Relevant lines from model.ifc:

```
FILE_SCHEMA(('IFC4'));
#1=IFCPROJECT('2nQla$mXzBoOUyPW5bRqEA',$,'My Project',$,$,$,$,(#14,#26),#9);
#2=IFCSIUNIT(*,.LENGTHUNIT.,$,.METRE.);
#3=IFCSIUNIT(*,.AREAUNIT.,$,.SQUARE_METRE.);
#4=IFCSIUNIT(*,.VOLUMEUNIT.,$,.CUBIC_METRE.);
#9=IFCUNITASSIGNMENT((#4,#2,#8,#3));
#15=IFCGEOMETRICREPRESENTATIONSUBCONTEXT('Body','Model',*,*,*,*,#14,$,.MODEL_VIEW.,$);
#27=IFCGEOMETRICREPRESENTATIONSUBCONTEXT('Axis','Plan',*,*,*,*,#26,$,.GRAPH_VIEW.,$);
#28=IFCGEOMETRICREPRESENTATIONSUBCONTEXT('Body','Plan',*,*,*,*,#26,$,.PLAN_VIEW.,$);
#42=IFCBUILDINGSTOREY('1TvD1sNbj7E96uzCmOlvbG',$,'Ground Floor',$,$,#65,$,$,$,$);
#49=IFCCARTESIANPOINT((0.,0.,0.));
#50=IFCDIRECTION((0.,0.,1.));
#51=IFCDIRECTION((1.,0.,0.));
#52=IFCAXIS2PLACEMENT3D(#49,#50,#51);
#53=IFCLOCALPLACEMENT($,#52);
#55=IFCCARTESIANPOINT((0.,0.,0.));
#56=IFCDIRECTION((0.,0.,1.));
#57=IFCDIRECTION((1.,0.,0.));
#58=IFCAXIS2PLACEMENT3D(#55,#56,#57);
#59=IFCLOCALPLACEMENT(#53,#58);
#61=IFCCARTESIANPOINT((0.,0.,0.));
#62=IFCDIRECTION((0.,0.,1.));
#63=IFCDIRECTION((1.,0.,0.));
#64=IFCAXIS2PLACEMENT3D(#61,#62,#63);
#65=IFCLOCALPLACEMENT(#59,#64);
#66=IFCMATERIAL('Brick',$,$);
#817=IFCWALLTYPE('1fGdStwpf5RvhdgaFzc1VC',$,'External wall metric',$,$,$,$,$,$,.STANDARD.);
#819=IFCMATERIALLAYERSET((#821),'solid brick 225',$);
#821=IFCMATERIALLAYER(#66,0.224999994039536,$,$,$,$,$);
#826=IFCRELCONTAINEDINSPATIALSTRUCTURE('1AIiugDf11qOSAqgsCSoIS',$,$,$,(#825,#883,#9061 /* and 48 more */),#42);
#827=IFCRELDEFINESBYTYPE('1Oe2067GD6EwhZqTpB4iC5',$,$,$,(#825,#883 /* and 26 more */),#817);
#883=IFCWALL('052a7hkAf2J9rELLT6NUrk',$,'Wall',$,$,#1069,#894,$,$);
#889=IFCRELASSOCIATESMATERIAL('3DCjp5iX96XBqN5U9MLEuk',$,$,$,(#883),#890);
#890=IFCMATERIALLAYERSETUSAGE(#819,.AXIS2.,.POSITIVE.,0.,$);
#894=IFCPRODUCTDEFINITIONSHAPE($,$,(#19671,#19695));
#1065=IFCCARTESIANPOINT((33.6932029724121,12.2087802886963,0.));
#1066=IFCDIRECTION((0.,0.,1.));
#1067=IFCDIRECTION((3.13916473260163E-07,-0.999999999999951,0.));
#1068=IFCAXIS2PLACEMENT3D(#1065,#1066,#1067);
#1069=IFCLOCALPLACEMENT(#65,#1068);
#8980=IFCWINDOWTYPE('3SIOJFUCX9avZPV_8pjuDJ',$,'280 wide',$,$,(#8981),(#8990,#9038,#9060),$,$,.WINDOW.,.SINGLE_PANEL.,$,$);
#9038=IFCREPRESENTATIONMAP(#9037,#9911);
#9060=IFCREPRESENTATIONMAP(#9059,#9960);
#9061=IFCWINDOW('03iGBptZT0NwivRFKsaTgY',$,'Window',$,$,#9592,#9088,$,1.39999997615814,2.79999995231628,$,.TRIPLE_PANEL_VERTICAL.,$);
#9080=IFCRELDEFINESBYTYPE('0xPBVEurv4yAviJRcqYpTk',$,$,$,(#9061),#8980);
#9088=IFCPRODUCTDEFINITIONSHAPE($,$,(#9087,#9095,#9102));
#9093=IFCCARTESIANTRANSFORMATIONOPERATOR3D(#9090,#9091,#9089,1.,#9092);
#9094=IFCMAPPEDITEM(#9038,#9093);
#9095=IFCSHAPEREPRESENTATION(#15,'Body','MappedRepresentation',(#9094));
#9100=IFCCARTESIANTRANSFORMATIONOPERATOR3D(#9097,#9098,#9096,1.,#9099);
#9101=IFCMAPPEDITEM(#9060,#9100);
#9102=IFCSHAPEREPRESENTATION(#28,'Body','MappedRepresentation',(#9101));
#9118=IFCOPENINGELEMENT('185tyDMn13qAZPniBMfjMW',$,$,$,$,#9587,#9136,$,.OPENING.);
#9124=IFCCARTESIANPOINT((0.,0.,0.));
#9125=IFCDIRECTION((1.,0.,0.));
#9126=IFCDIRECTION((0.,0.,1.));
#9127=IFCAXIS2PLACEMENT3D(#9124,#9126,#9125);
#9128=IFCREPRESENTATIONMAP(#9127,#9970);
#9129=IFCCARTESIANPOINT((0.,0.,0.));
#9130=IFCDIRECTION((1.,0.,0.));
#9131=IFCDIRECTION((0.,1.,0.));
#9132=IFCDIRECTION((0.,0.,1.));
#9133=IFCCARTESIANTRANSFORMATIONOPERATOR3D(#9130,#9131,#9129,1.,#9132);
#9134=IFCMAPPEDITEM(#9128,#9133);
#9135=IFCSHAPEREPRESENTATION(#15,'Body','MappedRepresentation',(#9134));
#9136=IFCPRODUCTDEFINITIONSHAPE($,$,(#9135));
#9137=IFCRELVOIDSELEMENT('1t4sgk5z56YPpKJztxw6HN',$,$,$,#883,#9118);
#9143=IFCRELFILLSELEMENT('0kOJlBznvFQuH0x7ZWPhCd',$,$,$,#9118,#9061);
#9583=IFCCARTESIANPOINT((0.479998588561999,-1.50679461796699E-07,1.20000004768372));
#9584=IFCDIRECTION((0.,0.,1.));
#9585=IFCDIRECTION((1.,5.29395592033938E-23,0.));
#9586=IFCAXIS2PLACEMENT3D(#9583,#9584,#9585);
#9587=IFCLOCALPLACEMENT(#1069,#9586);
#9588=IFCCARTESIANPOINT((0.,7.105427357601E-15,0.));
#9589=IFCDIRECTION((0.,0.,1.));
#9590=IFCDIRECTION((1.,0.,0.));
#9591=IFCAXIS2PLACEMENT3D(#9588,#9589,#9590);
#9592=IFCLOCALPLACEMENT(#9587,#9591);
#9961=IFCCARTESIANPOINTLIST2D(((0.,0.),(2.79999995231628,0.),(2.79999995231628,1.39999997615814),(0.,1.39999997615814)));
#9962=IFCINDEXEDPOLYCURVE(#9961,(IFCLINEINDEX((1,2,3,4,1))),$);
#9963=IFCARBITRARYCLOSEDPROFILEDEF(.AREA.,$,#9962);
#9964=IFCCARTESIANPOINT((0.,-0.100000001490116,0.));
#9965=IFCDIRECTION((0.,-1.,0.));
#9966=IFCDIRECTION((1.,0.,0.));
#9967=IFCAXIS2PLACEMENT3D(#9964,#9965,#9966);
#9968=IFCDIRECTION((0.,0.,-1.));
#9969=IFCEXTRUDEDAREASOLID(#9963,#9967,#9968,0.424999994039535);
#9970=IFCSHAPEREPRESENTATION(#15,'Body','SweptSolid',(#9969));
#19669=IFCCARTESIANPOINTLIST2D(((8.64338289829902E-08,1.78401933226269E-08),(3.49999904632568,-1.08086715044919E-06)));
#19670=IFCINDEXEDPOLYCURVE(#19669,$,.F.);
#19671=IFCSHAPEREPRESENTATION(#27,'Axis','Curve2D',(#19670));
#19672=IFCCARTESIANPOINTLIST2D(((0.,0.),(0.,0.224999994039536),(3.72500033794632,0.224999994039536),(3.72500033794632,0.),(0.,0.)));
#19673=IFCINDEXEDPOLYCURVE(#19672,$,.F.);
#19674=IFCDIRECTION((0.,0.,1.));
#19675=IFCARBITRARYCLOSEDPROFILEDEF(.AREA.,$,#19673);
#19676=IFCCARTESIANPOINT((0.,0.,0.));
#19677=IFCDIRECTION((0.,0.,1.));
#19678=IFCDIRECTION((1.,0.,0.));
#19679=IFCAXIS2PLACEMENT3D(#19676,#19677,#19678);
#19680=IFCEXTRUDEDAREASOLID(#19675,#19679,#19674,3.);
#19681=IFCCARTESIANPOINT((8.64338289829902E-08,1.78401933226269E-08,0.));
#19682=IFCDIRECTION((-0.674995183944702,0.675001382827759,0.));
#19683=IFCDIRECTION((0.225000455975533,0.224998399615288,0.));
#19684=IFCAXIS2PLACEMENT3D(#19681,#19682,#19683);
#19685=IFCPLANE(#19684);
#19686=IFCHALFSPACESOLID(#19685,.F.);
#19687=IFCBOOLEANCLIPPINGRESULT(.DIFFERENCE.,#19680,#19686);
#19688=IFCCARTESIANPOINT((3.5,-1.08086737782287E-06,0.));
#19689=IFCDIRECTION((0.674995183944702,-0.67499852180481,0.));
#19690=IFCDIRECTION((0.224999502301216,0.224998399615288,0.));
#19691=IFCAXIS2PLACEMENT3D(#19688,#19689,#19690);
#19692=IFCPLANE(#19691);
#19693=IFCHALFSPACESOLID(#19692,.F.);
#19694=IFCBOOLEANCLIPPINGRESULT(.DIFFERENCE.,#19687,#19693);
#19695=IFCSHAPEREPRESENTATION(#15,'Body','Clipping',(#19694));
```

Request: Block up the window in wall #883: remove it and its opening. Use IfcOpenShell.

```python
import ifcopenshell
import ifcopenshell.api.feature
import ifcopenshell.api.root
import ifcopenshell.geom
import ifcopenshell.util.shape

model = ifcopenshell.open("model.ifc")
settings = ifcopenshell.geom.settings()


def volume(element):
    """Net volume in cubic metres, openings subtracted."""
    shape = ifcopenshell.geom.create_shape(settings, element)
    return ifcopenshell.util.shape.get_volume(shape.geometry)


window = model.by_guid("03iGBptZT0NwivRFKsaTgY")
opening = window.FillsVoids[0].RelatingOpeningElement
wall = opening.VoidsElements[0].RelatingBuildingElement
before = volume(wall)

ifcopenshell.api.root.remove_product(model, product=window)
ifcopenshell.api.feature.remove_feature(model, feature=opening)

after = volume(wall)

print(f"wall volume {before:.3f} -> {after:.3f} m3")

model.write("model_updated.ifc")
```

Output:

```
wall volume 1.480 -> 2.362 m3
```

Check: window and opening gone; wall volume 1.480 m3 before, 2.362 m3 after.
